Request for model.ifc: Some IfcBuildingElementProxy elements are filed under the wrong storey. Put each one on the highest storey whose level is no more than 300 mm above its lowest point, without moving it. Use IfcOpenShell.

First a look at what the model holds.

```python
import ifcopenshell
import ifcopenshell.util.element
import ifcopenshell.util.placement

model = ifcopenshell.open("model.ifc")
print(model.schema)
for storey in model.by_type("IfcBuildingStorey"):
    level = ifcopenshell.util.placement.get_storey_elevation(storey)
    count = sum(e.is_a("IfcBuildingElementProxy") for e in ifcopenshell.util.element.get_contained(storey))
    print(storey.id(), storey.Name, round(level, 3), count, sep=" | ")
```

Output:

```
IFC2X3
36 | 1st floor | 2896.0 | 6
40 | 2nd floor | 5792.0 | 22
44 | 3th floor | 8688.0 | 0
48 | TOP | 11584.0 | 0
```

```python
import ifcopenshell
import ifcopenshell.api.spatial
import ifcopenshell.geom
import ifcopenshell.util.element
import ifcopenshell.util.placement
import ifcopenshell.util.shape
import ifcopenshell.util.unit

model = ifcopenshell.open("model.ifc")
unit_scale = ifcopenshell.util.unit.calculate_unit_scale(model)
settings = ifcopenshell.geom.settings()

levels = sorted(
    ((ifcopenshell.util.placement.get_storey_elevation(s) * unit_scale, s) for s in model.by_type("IfcBuildingStorey")),
    key=lambda pair: pair[0],
)

for e in model.by_type("IfcBuildingElementProxy"):
    current = e.ContainedInStructure[0].RelatingStructure if e.ContainedInStructure else None
    if current is None or not current.is_a("IfcBuildingStorey"):
        continue
    shape = ifcopenshell.geom.create_shape(settings, e)
    bottom = ifcopenshell.util.shape.get_shape_bottom_elevation(shape, shape.geometry)
    below = [s for level, s in levels if level <= bottom + 0.3]
    storey = below[-1] if below else levels[0][1]
    if storey != current:
        # assign_container keeps the world position.
        ifcopenshell.api.spatial.assign_container(model, products=[e], relating_structure=storey)
        print(e.id(), current.Name, "->", storey.Name)

model.write("model_edited.ifc")
```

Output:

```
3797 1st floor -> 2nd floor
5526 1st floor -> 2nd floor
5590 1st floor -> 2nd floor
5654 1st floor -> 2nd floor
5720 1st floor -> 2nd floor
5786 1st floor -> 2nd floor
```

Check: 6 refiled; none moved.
